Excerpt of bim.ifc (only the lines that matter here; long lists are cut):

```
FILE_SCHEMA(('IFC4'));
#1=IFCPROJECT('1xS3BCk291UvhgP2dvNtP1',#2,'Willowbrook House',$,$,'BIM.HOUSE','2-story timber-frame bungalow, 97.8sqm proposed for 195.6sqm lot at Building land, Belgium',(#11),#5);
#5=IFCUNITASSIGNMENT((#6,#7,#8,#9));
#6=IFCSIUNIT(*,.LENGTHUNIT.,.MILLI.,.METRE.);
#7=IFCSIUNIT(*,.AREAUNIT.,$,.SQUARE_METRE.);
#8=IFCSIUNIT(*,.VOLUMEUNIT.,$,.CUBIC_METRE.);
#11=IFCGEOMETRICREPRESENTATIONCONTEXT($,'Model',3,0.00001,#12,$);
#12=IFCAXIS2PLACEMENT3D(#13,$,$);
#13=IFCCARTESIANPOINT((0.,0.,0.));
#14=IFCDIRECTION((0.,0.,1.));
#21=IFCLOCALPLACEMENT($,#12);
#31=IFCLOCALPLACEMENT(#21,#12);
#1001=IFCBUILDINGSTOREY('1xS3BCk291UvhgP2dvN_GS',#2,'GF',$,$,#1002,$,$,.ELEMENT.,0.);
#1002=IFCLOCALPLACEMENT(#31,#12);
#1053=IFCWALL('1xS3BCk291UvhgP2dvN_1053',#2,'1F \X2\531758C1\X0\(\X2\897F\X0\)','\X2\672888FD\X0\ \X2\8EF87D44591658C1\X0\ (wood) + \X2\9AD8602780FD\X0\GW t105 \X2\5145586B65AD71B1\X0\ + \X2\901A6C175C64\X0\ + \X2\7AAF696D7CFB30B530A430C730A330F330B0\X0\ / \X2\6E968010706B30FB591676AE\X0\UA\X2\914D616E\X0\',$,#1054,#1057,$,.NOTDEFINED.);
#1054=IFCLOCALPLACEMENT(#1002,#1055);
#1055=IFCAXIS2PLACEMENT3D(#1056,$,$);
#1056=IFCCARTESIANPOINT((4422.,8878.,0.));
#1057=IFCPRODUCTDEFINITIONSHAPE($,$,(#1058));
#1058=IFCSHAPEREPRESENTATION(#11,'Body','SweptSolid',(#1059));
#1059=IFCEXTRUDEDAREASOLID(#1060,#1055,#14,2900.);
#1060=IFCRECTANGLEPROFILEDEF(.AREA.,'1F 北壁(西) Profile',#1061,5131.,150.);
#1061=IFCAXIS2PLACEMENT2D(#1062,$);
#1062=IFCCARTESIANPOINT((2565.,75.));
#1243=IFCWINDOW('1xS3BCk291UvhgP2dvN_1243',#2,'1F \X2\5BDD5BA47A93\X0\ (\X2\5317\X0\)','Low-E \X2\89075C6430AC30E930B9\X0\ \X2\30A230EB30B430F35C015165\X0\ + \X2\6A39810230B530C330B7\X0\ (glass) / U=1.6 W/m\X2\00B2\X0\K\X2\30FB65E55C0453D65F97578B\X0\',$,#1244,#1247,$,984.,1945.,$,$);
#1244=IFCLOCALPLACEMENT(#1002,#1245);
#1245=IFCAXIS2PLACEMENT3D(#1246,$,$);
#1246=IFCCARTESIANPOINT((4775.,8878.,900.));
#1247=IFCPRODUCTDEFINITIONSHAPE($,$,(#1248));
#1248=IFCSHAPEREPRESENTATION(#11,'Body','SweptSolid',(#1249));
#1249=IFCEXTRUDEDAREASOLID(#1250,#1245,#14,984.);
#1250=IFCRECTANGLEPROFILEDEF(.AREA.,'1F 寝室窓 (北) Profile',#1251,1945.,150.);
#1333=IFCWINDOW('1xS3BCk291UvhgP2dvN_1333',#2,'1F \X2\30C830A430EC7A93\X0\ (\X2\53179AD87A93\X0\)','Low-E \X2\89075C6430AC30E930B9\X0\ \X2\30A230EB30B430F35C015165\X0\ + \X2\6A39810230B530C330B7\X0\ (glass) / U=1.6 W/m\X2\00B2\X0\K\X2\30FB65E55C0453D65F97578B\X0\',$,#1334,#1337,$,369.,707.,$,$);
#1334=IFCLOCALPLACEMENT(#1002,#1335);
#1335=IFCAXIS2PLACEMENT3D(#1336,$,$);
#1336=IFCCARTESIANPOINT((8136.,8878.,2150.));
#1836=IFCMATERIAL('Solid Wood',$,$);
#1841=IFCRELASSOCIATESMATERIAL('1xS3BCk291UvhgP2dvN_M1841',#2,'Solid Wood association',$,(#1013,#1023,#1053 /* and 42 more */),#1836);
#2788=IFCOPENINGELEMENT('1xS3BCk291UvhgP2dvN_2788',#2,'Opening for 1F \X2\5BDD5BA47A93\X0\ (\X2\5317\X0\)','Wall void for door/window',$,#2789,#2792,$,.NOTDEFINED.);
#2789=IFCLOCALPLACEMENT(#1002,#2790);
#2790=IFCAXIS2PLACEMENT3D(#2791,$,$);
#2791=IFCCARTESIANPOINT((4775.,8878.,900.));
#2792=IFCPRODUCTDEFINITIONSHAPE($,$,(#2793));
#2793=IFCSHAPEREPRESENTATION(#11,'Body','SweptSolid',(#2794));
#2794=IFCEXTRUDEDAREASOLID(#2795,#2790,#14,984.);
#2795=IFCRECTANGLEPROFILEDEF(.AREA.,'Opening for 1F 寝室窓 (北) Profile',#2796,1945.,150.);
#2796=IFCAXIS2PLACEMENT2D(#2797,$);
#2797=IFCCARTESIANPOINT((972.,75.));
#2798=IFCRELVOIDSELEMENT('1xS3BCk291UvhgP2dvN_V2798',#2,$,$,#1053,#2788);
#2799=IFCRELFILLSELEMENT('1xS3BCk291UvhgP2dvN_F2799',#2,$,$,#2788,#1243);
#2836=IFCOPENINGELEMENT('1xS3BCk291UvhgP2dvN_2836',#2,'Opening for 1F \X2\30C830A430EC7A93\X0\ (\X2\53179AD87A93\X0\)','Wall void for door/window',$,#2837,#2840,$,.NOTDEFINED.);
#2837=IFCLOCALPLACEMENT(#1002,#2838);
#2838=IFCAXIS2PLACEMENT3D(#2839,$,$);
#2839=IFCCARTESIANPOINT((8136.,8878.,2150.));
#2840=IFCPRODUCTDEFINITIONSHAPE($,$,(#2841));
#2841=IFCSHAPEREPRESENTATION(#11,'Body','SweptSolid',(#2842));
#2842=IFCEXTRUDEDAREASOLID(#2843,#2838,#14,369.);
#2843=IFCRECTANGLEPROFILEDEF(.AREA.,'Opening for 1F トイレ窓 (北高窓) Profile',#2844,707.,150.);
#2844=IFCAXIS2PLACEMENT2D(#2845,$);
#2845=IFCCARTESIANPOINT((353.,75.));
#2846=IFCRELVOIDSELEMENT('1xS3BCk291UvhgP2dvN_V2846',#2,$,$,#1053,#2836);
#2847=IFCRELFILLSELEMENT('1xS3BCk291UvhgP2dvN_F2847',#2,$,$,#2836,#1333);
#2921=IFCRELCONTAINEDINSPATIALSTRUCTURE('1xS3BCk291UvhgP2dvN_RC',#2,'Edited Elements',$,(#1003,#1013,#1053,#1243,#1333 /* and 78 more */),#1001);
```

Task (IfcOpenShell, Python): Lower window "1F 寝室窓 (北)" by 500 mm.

```python
import numpy as np
import ifcopenshell
import ifcopenshell.api.geometry
import ifcopenshell.util.placement
import ifcopenshell.util.unit

model = ifcopenshell.open("bim.ifc")
unit_scale = ifcopenshell.util.unit.calculate_unit_scale(model)

window = model.by_guid("1xS3BCk291UvhgP2dvN_1243")
opening = window.FillsVoids[0].RelatingOpeningElement
dz = -500.0

shift = np.array([0.0, 0.0, dz])
# The window is not placed relative to its opening, so move both.
for product in (opening, window):
    matrix = ifcopenshell.util.placement.get_local_placement(product.ObjectPlacement)
    matrix[:3, 3] += shift
    ifcopenshell.api.geometry.edit_object_placement(model, product=product, matrix=matrix, is_si=False)

print(f"moved by {dz * unit_scale:+.3f} m")

model.write("bim_rev.ifc")
```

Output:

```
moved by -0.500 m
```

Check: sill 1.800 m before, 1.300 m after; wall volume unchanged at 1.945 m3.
